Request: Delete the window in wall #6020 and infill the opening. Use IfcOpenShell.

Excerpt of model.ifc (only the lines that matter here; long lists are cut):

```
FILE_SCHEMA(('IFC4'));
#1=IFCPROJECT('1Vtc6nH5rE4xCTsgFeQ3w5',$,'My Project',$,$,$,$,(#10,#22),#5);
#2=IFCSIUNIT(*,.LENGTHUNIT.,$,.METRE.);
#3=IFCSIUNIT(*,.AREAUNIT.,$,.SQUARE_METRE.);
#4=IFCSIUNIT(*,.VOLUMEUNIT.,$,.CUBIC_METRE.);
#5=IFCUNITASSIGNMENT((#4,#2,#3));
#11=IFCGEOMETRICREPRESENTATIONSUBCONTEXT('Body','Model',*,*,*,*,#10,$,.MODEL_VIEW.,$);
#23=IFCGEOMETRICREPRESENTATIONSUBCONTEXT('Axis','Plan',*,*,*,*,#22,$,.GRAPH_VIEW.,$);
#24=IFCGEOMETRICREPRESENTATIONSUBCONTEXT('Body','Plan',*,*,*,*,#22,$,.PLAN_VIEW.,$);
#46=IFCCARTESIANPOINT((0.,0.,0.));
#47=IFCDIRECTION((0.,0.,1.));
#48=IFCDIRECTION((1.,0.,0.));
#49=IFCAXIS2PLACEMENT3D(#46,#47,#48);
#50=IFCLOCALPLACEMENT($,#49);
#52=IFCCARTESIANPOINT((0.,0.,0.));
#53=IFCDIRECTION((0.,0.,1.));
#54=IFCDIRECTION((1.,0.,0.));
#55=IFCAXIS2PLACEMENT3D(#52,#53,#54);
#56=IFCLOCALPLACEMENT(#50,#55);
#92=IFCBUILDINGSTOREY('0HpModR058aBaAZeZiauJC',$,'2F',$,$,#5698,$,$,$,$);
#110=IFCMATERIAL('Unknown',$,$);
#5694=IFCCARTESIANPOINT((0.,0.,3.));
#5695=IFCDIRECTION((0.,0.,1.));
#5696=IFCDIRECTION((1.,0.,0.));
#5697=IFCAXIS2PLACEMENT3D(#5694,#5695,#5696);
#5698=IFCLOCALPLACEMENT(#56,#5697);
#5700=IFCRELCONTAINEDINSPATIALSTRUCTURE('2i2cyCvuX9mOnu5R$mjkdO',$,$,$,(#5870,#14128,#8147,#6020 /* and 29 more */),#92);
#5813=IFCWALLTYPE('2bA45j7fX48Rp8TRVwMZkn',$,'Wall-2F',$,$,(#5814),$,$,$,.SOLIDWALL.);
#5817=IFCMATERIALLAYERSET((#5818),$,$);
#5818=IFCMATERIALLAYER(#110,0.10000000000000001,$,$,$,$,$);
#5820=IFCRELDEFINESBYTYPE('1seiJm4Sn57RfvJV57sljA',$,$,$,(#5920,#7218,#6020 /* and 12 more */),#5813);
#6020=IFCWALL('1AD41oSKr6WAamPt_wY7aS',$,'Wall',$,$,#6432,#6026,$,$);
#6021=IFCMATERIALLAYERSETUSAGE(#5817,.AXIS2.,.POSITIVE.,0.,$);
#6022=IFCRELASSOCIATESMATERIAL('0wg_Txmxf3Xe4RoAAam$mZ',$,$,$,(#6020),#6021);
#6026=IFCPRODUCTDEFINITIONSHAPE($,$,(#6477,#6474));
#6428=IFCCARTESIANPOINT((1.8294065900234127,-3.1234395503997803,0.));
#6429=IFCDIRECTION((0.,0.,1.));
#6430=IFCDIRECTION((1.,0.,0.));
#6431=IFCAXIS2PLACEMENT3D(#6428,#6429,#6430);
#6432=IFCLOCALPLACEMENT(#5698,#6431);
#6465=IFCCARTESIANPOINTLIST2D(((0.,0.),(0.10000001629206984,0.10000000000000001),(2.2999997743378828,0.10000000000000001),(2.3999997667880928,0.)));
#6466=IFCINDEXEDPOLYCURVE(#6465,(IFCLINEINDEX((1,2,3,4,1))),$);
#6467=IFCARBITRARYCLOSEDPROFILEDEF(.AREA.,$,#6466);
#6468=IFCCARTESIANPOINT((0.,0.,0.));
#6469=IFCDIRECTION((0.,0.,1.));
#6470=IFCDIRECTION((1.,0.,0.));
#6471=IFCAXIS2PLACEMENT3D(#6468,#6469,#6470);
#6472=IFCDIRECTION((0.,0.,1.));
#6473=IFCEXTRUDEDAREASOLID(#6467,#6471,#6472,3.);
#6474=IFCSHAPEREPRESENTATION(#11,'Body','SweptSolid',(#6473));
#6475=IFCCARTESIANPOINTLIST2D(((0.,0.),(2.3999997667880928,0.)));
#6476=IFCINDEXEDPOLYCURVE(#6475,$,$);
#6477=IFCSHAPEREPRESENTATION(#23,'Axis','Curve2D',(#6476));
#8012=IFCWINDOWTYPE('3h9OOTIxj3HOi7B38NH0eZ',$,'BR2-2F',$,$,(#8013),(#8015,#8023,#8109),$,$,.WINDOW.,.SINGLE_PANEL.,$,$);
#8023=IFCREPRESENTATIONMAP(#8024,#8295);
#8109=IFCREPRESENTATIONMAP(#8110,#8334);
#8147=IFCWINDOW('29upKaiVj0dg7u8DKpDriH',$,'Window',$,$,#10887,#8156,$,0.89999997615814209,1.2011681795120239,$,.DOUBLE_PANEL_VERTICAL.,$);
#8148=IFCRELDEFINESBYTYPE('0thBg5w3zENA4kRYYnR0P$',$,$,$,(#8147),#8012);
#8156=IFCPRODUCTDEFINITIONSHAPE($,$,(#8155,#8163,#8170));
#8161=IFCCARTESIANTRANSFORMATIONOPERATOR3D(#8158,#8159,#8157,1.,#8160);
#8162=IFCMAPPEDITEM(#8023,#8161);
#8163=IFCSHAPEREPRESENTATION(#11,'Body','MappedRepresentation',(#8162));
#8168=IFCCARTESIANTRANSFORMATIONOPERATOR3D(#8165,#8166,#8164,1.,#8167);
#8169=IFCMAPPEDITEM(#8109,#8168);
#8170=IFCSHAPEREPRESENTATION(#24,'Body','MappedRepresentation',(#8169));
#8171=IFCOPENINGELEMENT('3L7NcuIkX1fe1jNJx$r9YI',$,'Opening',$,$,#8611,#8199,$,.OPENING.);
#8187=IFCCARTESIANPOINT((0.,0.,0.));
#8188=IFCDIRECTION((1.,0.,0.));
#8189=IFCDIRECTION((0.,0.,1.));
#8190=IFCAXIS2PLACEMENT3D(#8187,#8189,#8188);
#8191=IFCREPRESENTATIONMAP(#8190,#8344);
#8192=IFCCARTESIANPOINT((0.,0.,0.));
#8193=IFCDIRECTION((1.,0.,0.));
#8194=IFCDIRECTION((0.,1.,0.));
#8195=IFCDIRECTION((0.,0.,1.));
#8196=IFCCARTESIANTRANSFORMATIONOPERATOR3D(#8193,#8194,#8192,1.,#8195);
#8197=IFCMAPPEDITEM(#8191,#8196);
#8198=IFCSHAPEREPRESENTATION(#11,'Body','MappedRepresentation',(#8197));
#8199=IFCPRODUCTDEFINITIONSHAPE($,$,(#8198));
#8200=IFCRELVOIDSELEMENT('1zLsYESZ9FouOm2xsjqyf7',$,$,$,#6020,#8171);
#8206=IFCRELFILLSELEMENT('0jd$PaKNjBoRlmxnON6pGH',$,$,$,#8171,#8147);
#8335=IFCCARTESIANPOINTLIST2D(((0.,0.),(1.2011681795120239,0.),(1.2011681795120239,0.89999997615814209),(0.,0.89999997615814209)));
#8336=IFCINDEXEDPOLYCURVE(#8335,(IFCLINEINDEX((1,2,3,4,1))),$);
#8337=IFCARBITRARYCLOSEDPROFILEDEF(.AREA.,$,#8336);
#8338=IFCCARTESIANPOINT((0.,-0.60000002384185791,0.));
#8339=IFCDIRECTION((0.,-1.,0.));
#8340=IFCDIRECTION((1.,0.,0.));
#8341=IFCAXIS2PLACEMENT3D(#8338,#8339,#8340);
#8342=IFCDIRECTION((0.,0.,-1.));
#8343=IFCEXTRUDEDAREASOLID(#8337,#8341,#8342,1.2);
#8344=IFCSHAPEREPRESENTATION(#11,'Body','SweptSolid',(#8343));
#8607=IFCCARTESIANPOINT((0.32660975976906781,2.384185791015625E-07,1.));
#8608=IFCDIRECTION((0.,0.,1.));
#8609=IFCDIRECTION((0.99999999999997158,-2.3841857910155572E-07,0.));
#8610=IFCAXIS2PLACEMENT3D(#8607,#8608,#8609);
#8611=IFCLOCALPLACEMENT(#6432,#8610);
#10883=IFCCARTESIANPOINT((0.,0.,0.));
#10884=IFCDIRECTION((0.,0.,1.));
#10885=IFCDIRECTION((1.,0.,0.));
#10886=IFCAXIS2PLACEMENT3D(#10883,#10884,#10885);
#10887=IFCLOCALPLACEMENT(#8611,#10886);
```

```python
import ifcopenshell
import ifcopenshell.api.feature
import ifcopenshell.api.root
import ifcopenshell.geom
import ifcopenshell.util.shape

model = ifcopenshell.open("model.ifc")
settings = ifcopenshell.geom.settings()


def volume(element):
    """Net volume in cubic metres, openings subtracted."""
    shape = ifcopenshell.geom.create_shape(settings, element)
    return ifcopenshell.util.shape.get_volume(shape.geometry)


window = model.by_guid("29upKaiVj0dg7u8DKpDriH")
opening = window.FillsVoids[0].RelatingOpeningElement
wall = opening.VoidsElements[0].RelatingBuildingElement
before = volume(wall)

ifcopenshell.api.root.remove_product(model, product=window)
ifcopenshell.api.feature.remove_feature(model, feature=opening)

after = volume(wall)

print(f"wall volume {before:.3f} -> {after:.3f} m3")

model.write("model_v2.ifc")
```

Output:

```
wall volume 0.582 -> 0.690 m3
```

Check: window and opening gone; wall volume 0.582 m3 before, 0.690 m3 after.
